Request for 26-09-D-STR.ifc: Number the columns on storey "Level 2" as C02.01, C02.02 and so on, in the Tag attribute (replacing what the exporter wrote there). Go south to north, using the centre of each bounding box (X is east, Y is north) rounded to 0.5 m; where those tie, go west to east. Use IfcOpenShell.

First a look at what the model holds.

```python
import ifcopenshell
import ifcopenshell.util.element
import ifcopenshell.util.placement

model = ifcopenshell.open("26-09-D-STR.ifc")
print(model.schema)
storey = next(s for s in model.by_type("IfcBuildingStorey") if s.Name == "Level 2")
columns = [e for e in ifcopenshell.util.element.get_decomposition(storey) if e.is_a("IfcColumn")]
for e in sorted(columns, key=lambda e: e.id()):
    origin = ifcopenshell.util.placement.get_local_placement(e.ObjectPlacement)[:3, 3]
    print(e.id(), e.Tag, e.Name, origin.round(2) + 0.0, sep=" | ")
```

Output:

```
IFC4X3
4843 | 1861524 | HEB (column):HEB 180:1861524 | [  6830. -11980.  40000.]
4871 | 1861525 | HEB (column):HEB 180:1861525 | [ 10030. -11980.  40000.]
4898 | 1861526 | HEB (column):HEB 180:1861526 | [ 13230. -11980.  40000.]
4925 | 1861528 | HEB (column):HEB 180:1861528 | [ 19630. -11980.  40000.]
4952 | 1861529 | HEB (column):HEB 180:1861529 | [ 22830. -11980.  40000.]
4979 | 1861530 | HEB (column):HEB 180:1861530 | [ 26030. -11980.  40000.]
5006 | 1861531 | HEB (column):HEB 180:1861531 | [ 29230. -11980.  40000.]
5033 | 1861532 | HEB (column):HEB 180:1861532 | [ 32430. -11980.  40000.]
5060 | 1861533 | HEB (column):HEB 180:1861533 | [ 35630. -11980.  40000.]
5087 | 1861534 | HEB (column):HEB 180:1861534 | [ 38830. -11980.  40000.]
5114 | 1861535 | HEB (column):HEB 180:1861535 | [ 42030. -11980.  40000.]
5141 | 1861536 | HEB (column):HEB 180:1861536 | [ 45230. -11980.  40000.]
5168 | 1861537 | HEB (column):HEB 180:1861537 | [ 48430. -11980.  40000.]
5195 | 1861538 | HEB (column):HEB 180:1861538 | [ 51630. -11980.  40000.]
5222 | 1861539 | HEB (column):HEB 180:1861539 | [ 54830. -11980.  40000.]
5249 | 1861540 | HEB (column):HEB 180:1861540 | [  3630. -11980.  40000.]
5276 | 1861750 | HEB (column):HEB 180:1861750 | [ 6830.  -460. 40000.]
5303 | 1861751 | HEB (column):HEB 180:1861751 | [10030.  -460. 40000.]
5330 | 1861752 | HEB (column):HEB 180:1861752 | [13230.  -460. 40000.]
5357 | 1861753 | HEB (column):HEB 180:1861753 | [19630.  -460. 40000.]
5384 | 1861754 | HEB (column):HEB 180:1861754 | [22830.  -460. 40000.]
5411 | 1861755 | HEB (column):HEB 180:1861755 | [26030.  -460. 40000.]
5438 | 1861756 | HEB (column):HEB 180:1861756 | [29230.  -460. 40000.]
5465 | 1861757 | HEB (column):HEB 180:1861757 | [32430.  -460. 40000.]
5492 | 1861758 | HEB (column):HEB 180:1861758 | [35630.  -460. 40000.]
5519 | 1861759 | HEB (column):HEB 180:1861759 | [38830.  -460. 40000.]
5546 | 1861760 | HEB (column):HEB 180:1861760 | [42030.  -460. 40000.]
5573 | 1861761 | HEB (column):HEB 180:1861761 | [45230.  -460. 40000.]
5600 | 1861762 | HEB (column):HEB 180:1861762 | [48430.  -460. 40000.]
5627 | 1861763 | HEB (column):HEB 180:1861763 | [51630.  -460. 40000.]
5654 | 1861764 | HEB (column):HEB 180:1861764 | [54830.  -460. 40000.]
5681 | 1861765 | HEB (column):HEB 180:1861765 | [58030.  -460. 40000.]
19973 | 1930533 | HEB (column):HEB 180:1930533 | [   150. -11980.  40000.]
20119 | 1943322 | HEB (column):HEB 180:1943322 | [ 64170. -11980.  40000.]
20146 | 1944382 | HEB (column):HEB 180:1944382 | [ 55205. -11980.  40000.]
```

```python
import ifcopenshell
import ifcopenshell.geom
import ifcopenshell.util.element
import ifcopenshell.util.shape

model = ifcopenshell.open("26-09-D-STR.ifc")
settings = ifcopenshell.geom.settings()
settings.set("use-world-coords", True)


def centre(element):
    shape = ifcopenshell.geom.create_shape(settings, element)
    return ifcopenshell.util.shape.get_bbox_centroid(shape.geometry)


storey = next(s for s in model.by_type("IfcBuildingStorey") if s.Name == "Level 2")
columns = [e for e in ifcopenshell.util.element.get_decomposition(storey) if e.is_a("IfcColumn")]

# Insertion points can sit at a corner or the storey origin, so sort by the geometry (in metres).
centres = {e: centre(e) for e in columns}
columns.sort(key=lambda e: (round(centres[e][1] / 0.5), centres[e][0]))

for i, e in enumerate(columns, start=1):
    number = f"C02.{i:02d}"
    e.Tag = number
    print(e.id(), number)

model.write("26-09-D-STR_updated.ifc")
```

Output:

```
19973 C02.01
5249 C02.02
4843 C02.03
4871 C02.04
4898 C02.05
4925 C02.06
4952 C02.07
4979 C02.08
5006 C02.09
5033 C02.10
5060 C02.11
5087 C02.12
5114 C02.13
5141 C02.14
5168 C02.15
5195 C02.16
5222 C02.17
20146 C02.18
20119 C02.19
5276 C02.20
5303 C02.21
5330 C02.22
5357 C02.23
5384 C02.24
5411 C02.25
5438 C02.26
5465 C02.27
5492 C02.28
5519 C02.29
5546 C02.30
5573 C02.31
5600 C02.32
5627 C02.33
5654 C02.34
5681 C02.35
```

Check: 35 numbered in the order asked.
